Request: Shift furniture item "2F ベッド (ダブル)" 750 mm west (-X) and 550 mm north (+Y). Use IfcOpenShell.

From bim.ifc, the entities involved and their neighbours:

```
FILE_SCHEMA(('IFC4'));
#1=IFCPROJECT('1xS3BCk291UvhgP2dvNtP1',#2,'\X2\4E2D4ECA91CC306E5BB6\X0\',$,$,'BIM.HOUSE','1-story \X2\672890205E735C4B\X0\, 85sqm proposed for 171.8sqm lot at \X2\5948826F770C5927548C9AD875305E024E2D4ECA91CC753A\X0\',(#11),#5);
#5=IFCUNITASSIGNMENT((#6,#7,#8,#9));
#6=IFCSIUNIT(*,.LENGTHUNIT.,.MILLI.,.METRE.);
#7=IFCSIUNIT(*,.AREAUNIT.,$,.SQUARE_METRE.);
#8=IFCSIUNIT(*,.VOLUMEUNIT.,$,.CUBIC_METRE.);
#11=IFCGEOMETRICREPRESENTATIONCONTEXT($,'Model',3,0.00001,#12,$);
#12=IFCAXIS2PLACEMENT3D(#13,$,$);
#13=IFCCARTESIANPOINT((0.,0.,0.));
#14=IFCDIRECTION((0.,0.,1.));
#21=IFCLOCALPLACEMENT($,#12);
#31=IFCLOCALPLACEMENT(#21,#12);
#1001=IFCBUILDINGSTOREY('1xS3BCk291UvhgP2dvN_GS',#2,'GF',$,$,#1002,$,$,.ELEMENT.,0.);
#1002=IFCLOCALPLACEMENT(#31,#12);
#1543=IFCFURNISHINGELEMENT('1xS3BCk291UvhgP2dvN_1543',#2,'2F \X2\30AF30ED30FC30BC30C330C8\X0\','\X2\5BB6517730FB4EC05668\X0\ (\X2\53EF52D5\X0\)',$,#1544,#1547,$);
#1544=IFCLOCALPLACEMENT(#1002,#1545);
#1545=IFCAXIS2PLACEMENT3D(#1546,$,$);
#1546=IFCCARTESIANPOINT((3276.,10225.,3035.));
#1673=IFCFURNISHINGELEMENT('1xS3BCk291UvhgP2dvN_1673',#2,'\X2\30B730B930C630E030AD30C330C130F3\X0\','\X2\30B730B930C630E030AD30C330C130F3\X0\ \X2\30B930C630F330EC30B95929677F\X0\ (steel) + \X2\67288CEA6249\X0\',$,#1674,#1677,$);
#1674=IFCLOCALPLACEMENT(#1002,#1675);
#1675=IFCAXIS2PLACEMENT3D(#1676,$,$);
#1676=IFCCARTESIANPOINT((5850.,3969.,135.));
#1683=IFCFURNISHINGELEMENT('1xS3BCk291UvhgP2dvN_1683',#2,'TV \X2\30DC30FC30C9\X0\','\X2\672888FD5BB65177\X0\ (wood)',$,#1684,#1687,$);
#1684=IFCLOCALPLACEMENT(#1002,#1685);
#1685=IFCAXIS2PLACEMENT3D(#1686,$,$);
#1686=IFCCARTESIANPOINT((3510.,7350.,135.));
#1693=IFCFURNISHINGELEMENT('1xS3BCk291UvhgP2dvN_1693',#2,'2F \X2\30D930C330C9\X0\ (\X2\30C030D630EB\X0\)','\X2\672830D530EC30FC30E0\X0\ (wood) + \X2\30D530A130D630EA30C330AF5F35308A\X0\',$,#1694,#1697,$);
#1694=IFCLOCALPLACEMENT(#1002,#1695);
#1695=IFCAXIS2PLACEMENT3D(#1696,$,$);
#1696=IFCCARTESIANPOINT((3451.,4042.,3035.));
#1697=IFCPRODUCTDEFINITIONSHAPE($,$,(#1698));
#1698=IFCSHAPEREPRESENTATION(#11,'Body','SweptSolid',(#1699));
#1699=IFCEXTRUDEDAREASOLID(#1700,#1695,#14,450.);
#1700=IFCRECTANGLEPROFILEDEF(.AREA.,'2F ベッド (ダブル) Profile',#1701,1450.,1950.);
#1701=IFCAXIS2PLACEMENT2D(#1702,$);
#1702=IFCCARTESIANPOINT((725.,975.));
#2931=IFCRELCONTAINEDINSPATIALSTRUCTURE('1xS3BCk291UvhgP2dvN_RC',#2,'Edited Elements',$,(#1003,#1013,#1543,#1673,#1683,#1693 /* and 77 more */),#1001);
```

```python
import ifcopenshell
import ifcopenshell.api.geometry
import ifcopenshell.util.placement

model = ifcopenshell.open("bim.ifc")

item = model.by_id(1693)
matrix = ifcopenshell.util.placement.get_local_placement(item.ObjectPlacement)
matrix[0, 3] -= 750.0
matrix[1, 3] += 550.0
ifcopenshell.api.geometry.edit_object_placement(model, product=item, matrix=matrix, is_si=False)

print(ifcopenshell.util.placement.get_local_placement(item.ObjectPlacement).round(3) + 0.0)

model.write("bim_rev.ifc")
```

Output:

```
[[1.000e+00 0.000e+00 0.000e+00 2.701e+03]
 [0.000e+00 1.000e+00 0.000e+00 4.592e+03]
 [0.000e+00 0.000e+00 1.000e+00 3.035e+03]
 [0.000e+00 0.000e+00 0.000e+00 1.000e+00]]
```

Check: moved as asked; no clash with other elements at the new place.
